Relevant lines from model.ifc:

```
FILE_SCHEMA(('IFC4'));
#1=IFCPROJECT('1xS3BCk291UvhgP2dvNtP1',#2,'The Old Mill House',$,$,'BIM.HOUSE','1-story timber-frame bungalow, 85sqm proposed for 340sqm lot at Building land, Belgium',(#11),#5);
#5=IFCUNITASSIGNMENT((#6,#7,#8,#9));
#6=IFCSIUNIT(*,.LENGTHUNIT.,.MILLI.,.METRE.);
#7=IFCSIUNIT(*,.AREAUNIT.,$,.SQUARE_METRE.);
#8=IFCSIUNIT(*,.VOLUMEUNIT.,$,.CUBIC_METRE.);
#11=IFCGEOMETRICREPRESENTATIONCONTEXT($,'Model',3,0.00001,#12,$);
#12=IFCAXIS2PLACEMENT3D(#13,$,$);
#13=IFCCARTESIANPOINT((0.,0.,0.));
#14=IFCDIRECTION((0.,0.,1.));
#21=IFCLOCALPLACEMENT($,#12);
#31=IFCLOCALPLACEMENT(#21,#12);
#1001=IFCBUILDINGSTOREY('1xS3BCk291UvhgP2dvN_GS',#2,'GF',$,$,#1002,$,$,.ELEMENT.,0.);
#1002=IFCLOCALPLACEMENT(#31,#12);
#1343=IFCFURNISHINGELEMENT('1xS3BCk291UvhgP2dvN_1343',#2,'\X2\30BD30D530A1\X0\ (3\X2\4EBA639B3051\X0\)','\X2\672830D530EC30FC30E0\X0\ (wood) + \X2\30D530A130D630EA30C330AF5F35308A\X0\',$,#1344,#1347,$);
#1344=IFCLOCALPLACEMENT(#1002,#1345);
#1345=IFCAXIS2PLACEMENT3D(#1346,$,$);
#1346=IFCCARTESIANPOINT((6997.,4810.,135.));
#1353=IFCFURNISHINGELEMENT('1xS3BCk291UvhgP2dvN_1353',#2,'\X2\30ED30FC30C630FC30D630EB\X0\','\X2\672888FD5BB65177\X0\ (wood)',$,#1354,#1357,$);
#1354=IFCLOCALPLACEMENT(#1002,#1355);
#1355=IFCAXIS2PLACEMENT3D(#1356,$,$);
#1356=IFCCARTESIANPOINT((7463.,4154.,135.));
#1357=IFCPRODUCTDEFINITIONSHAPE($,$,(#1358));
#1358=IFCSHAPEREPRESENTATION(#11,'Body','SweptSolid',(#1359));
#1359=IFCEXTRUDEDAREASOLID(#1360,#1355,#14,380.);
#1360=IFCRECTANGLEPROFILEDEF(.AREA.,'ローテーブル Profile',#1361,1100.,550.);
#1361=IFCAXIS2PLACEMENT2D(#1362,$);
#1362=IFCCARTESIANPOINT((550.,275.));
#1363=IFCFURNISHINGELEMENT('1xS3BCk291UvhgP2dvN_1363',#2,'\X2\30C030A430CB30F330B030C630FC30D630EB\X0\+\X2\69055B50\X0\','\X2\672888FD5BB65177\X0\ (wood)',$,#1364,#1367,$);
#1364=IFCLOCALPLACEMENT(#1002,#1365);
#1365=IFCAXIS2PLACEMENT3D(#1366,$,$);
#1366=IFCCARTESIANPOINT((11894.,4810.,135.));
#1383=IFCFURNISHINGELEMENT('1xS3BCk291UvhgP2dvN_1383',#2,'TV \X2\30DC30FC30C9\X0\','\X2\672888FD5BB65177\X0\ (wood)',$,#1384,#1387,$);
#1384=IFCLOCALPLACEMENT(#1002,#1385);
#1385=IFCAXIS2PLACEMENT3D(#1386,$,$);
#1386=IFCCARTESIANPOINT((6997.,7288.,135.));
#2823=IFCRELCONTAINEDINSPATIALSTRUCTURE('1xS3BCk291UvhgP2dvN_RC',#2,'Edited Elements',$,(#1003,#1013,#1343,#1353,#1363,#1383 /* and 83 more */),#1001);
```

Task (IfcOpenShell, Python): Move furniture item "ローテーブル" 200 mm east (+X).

```python
import ifcopenshell
import ifcopenshell.api.geometry
import ifcopenshell.util.placement
import ifcopenshell.util.unit

model = ifcopenshell.open("model.ifc")
unit_scale = ifcopenshell.util.unit.calculate_unit_scale(model)

item = model.by_guid("1xS3BCk291UvhgP2dvN_1353")
matrix = ifcopenshell.util.placement.get_local_placement(item.ObjectPlacement)
matrix[0, 3] += 0.2 / unit_scale
ifcopenshell.api.geometry.edit_object_placement(model, product=item, matrix=matrix, is_si=False)

print(ifcopenshell.util.placement.get_local_placement(item.ObjectPlacement).round(3) + 0.0)

model.write("model_updated.ifc")
```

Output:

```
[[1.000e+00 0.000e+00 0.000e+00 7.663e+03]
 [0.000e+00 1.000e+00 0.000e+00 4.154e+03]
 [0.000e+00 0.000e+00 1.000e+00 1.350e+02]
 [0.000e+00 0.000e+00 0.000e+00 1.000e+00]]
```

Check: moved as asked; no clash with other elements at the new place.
